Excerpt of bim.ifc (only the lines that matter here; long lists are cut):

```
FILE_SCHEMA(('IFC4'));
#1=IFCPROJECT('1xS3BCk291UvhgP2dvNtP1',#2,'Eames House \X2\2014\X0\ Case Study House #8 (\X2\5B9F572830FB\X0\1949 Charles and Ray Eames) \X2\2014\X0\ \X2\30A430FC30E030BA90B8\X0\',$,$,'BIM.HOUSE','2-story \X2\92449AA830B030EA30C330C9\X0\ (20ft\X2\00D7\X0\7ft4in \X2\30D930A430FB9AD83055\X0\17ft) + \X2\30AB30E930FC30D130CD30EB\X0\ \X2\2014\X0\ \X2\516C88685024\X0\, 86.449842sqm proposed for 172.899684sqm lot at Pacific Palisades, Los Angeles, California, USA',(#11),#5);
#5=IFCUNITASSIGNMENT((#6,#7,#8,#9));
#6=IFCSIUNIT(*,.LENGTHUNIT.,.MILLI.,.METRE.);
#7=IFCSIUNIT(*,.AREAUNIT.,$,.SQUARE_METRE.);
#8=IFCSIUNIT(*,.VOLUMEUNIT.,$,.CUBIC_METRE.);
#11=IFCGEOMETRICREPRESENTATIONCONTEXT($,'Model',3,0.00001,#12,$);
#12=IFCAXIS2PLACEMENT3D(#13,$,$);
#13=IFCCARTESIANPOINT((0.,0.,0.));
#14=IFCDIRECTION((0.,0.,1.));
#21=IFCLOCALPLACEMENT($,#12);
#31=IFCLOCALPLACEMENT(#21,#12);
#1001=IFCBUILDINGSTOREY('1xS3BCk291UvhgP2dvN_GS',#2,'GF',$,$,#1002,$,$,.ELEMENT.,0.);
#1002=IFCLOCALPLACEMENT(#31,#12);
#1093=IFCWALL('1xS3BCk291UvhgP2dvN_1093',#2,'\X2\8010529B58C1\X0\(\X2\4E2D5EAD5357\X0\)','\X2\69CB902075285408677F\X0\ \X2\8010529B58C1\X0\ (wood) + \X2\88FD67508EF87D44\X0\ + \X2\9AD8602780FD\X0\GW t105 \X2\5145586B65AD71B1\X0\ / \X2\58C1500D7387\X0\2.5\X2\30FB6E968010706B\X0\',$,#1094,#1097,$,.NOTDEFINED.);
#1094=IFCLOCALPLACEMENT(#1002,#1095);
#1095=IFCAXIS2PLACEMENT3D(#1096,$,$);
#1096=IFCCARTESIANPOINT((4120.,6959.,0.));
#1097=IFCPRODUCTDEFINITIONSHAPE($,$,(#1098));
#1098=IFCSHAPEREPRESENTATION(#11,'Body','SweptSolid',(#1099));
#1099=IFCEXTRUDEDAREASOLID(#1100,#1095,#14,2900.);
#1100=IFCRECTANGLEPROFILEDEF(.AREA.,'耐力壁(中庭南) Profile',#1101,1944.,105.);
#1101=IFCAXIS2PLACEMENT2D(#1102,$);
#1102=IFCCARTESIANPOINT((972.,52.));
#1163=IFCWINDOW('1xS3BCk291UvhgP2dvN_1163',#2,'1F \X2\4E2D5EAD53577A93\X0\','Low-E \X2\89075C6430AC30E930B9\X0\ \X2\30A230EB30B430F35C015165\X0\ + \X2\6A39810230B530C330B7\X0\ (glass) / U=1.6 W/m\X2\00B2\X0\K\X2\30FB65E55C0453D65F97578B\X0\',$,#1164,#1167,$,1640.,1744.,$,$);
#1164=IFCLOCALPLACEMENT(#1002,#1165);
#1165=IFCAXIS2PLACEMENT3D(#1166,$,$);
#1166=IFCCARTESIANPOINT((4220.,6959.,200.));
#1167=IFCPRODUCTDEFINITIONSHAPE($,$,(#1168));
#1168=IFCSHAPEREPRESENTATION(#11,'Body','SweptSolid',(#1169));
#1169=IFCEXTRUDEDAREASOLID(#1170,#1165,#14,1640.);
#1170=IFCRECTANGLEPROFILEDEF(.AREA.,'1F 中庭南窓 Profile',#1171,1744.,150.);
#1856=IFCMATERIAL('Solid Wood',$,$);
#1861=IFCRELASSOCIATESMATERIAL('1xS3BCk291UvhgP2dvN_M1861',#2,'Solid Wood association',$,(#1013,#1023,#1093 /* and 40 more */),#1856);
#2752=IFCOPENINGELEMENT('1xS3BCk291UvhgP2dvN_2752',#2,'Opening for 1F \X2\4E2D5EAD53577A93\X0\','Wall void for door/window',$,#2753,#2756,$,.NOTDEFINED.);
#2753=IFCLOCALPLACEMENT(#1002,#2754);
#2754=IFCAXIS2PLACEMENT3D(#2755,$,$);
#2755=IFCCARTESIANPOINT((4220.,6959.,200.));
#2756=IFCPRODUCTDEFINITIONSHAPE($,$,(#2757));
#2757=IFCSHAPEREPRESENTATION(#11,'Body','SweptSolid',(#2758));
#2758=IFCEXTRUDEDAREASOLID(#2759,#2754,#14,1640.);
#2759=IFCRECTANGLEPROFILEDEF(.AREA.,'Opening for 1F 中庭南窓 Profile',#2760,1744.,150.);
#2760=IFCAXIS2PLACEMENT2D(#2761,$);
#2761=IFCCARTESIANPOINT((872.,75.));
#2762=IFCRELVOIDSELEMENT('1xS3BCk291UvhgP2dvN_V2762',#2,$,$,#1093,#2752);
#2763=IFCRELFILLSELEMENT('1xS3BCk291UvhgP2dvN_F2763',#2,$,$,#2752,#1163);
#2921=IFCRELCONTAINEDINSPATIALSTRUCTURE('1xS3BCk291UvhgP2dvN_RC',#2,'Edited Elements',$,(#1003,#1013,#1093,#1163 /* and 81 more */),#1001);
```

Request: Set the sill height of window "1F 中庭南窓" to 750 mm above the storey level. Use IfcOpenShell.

```python
import numpy as np
import ifcopenshell
import ifcopenshell.api.geometry
import ifcopenshell.geom
import ifcopenshell.util.element
import ifcopenshell.util.placement
import ifcopenshell.util.shape
import ifcopenshell.util.unit

model = ifcopenshell.open("bim.ifc")
unit_scale = ifcopenshell.util.unit.calculate_unit_scale(model)

window = model.by_guid("1xS3BCk291UvhgP2dvN_1163")
opening = window.FillsVoids[0].RelatingOpeningElement
storey = ifcopenshell.util.element.get_container(window, ifc_class="IfcBuildingStorey")
level = ifcopenshell.util.placement.get_local_placement(storey.ObjectPlacement)[2, 3]

# The opening's origin need not be at the sill, so measure its lowest point.
shape = ifcopenshell.geom.create_shape(ifcopenshell.geom.settings(), opening)
bottom = ifcopenshell.util.shape.get_shape_bottom_elevation(shape, shape.geometry) / unit_scale
dz = level + 750.0 - bottom

shift = np.array([0.0, 0.0, dz])
# The window is not placed relative to its opening, so move both.
for product in (opening, window):
    matrix = ifcopenshell.util.placement.get_local_placement(product.ObjectPlacement)
    matrix[:3, 3] += shift
    ifcopenshell.api.geometry.edit_object_placement(model, product=product, matrix=matrix, is_si=False)

print(f"moved by {dz * unit_scale:+.3f} m")

model.write("bim_edited.ifc")
```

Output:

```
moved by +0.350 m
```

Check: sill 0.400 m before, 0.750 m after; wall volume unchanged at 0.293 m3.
